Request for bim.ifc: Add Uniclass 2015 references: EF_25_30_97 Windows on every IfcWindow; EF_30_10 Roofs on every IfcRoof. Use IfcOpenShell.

First a look at what the model holds.

```python
import ifcopenshell

model = ifcopenshell.open("bim.ifc")
print(model.schema)
print("classifications:", [c.Name for c in model.by_type("IfcClassification")])
for ifc_class in ("IfcDoor", "IfcRoof", "IfcStair", "IfcWall", "IfcWindow"):
    print(ifc_class, len(model.by_type(ifc_class)))
```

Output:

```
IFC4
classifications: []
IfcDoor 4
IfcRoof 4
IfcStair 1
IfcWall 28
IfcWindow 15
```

```python
import ifcopenshell
import ifcopenshell.api.classification

model = ifcopenshell.open("bim.ifc")

system = ifcopenshell.api.classification.add_classification(model, classification="Uniclass 2015")

codes = {
    "IfcWindow": ("EF_25_30_97", "Windows"),
    "IfcRoof": ("EF_30_10", "Roofs"),
}
for ifc_class, (code, name) in codes.items():
    products = model.by_type(ifc_class)
    ifcopenshell.api.classification.add_reference(
        model, products=products, classification=system, identification=code, name=name
    )
    print(code, len(products))

model.write("bim_v2.ifc")
```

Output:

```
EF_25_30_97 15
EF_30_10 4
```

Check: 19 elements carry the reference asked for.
